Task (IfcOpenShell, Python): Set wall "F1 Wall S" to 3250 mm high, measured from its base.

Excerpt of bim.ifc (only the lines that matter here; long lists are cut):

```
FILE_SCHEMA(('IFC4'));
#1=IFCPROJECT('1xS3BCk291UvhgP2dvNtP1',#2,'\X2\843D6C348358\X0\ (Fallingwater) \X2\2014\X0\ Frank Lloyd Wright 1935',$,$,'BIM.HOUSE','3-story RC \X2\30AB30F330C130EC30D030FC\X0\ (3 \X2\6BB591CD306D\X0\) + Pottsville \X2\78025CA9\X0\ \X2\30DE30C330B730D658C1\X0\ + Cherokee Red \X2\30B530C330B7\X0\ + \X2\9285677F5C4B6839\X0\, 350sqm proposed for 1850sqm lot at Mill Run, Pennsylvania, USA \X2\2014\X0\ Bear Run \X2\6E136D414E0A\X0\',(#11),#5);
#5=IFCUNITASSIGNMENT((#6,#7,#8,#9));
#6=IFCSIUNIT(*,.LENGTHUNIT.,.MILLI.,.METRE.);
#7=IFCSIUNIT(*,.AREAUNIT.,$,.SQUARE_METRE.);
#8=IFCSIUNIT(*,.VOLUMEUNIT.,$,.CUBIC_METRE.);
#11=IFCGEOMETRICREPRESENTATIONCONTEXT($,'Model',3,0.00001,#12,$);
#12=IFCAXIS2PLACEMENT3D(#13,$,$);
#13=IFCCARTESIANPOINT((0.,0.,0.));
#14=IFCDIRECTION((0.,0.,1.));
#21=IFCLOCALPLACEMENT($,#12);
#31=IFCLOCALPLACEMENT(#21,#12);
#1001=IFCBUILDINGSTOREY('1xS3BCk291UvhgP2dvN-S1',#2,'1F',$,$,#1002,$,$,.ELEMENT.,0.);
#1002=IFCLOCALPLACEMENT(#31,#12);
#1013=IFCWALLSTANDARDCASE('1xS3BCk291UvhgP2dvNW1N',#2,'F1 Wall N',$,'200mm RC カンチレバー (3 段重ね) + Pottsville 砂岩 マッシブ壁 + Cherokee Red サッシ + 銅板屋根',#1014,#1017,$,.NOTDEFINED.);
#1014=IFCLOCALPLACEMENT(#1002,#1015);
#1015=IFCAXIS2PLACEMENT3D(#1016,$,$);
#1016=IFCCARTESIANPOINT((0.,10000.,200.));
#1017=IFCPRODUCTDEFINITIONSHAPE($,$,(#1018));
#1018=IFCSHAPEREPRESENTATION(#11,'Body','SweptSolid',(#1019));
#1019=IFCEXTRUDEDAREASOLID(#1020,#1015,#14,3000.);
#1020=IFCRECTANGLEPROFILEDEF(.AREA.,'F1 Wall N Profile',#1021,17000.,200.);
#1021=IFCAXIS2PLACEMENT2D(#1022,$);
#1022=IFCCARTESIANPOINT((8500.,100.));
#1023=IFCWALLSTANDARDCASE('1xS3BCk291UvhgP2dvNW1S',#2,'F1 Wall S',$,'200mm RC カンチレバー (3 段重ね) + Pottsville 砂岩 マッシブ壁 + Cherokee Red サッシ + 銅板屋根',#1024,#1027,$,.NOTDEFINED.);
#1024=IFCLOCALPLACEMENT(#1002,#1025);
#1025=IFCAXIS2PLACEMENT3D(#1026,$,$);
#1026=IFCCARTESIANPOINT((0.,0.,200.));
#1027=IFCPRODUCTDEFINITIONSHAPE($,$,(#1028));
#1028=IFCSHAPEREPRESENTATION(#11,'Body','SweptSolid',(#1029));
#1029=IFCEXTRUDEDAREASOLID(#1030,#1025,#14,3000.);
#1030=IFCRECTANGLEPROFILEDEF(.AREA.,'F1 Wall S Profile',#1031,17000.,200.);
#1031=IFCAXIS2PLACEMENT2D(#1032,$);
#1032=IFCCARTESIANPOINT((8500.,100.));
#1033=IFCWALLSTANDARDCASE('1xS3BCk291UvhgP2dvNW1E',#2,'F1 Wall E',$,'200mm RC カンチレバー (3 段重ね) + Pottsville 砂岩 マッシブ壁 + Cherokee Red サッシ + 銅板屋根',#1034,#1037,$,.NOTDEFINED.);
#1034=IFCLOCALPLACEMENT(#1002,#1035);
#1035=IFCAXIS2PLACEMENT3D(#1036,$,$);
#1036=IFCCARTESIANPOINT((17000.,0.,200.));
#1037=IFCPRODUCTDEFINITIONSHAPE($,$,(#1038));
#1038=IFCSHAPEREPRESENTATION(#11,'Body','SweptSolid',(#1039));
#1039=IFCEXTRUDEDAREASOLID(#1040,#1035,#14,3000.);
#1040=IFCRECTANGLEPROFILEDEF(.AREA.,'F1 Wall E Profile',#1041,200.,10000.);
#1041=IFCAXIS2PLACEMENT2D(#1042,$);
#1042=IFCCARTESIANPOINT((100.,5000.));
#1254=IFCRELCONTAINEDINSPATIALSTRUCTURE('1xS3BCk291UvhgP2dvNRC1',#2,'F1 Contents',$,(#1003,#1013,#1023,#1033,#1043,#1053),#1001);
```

```python
import ifcopenshell
import ifcopenshell.geom
import ifcopenshell.util.shape
import ifcopenshell.util.unit

model = ifcopenshell.open("bim.ifc")
unit_scale = ifcopenshell.util.unit.calculate_unit_scale(model)
settings = ifcopenshell.geom.settings()


def volume(element):
    """Net volume in cubic metres, openings subtracted."""
    shape = ifcopenshell.geom.create_shape(settings, element)
    return ifcopenshell.util.shape.get_volume(shape.geometry)


wall = model.by_guid("1xS3BCk291UvhgP2dvNW1S")
before = volume(wall)

body = next(r for r in wall.Representation.Representations if r.RepresentationIdentifier == "Body")
solid = body.Items[0]
old_height = solid.Depth
solid.Depth = 3.25 / unit_scale
after = volume(wall)

print(f"height {old_height:g} -> {solid.Depth:g}, volume {before:.3f} -> {after:.3f} m3")

model.write("bim-out.ifc")
```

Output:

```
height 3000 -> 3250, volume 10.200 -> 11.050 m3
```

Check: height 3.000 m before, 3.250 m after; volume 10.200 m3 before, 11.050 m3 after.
